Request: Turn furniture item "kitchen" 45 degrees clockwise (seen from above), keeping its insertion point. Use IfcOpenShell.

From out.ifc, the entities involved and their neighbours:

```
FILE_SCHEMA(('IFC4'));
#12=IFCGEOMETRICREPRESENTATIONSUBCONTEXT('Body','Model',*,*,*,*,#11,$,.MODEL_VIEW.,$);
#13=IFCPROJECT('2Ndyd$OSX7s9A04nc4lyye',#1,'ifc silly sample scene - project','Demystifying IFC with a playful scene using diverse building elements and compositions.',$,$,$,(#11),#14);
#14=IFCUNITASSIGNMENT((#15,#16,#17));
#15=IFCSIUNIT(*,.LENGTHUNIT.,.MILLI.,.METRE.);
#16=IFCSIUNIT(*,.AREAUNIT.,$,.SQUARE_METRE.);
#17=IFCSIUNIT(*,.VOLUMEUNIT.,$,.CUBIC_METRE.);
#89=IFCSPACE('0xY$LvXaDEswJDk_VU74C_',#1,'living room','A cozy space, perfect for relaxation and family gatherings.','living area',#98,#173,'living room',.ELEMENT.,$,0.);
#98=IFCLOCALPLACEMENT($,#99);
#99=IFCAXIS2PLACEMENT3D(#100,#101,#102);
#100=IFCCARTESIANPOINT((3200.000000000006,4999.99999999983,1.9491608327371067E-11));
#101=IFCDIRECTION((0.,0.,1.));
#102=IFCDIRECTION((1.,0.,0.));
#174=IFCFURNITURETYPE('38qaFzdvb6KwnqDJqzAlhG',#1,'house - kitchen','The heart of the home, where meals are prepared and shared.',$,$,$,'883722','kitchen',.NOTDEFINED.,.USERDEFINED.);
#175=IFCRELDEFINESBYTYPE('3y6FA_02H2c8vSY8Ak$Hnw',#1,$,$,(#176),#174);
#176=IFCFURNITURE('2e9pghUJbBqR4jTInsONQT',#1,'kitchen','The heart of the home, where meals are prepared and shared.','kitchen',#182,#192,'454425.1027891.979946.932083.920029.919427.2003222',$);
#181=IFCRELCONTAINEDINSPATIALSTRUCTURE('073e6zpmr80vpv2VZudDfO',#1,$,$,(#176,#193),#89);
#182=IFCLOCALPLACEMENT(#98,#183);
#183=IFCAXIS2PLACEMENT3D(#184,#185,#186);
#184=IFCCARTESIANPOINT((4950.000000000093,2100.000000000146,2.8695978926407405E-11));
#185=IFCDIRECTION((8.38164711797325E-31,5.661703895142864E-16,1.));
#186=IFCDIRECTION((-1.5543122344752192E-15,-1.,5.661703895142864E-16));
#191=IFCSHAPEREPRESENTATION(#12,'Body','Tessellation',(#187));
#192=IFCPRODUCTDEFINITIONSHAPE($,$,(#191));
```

```python
import ifcopenshell
import ifcopenshell.api.geometry
import ifcopenshell.util.placement

model = ifcopenshell.open("out.ifc")

item = model.by_id(176)
matrix = ifcopenshell.util.placement.get_local_placement(item.ObjectPlacement)
matrix = matrix @ ifcopenshell.util.placement.rotation(-45, "Z")
ifcopenshell.api.geometry.edit_object_placement(model, product=item, matrix=matrix, is_si=False)

print(ifcopenshell.util.placement.get_local_placement(item.ObjectPlacement).round(3) + 0.0)

model.write("out_rev.ifc")
```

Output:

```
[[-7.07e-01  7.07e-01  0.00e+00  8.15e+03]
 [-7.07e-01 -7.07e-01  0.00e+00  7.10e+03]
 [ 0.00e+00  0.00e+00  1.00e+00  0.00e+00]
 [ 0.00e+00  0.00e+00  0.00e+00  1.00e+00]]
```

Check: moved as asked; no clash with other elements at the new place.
